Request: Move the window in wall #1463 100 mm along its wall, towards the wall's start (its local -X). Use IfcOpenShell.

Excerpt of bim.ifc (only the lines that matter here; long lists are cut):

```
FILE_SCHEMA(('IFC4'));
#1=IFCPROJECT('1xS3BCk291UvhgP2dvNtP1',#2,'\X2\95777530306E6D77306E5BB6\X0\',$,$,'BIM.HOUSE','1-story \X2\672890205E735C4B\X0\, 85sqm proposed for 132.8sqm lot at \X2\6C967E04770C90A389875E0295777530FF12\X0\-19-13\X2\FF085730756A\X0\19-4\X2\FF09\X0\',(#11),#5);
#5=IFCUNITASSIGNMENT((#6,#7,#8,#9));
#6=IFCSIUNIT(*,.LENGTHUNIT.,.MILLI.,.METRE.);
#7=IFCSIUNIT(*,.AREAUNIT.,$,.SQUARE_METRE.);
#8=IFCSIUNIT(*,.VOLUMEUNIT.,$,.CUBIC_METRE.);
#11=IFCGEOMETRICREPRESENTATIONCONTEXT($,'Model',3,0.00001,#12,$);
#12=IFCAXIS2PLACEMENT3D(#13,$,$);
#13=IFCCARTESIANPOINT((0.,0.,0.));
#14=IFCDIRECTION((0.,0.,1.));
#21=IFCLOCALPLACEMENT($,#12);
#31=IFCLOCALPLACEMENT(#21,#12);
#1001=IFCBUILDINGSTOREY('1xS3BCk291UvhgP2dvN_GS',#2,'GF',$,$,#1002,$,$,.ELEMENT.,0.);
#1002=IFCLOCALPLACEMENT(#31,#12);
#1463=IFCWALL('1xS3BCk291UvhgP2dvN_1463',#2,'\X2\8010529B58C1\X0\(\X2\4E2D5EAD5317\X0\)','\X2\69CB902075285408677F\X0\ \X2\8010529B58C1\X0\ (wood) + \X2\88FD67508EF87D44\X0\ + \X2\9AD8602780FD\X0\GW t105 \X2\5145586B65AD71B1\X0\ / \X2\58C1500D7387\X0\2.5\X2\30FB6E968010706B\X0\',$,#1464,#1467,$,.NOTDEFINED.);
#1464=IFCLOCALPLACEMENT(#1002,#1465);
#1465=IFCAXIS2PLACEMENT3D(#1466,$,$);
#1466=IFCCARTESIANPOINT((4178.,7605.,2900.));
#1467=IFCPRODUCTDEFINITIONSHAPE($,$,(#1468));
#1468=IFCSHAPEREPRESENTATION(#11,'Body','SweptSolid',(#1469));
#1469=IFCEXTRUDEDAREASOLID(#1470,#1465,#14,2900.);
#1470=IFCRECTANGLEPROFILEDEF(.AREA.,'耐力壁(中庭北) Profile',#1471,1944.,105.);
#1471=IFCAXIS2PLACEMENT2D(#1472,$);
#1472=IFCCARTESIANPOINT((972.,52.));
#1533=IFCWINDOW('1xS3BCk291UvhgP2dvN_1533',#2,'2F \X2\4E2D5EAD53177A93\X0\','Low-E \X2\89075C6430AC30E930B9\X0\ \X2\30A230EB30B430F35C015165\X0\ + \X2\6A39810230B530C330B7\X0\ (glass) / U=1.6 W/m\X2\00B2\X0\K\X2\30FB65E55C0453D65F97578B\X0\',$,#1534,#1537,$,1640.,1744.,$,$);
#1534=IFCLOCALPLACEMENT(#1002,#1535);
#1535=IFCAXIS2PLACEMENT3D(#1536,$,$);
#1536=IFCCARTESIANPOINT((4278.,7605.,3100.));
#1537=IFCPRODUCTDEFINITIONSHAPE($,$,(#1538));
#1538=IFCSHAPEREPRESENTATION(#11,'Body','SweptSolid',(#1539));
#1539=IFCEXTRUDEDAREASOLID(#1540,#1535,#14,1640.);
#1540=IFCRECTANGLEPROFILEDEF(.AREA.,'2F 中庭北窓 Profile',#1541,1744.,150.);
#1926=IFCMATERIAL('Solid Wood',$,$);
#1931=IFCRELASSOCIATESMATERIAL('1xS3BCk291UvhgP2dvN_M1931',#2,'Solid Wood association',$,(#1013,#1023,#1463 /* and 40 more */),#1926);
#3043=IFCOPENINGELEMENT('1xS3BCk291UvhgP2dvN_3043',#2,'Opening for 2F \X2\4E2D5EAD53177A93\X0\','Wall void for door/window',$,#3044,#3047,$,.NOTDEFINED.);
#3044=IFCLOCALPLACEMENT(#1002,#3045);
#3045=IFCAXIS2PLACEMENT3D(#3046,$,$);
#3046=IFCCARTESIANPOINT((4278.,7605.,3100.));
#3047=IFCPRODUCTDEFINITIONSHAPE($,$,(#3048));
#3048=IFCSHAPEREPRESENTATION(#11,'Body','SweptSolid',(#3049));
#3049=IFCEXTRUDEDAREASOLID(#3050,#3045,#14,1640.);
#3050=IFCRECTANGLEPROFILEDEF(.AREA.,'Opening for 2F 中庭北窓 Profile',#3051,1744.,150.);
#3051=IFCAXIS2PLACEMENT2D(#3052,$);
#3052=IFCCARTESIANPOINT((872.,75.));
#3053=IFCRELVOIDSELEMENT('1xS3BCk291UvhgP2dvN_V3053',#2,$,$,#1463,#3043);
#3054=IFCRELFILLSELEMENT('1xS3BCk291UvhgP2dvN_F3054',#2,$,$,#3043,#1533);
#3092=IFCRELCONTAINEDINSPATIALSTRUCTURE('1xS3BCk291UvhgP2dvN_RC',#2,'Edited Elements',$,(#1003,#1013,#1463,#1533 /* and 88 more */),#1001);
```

```python
import ifcopenshell
import ifcopenshell.api.geometry
import ifcopenshell.util.placement

model = ifcopenshell.open("bim.ifc")

window = model.by_guid("1xS3BCk291UvhgP2dvN_1533")
opening = window.FillsVoids[0].RelatingOpeningElement
wall = opening.VoidsElements[0].RelatingBuildingElement

wall_matrix = ifcopenshell.util.placement.get_local_placement(wall.ObjectPlacement)
shift = wall_matrix[:3, 0] * -100.0
before = ifcopenshell.util.placement.get_local_placement(window.ObjectPlacement)[:3, 3].copy()

# The window is not placed relative to its opening, so move both.
for product in (opening, window):
    matrix = ifcopenshell.util.placement.get_local_placement(product.ObjectPlacement)
    matrix[:3, 3] += shift
    ifcopenshell.api.geometry.edit_object_placement(model, product=product, matrix=matrix, is_si=False)

after = ifcopenshell.util.placement.get_local_placement(window.ObjectPlacement)[:3, 3]
print("window moved by", (after - before).round(3) + 0.0)

model.write("bim-out.ifc")
```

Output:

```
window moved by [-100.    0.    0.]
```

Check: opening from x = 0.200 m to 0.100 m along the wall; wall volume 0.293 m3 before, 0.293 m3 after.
